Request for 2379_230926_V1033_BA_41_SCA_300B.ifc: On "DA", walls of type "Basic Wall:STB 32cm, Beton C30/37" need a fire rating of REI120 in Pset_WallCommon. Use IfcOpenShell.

First a look at what the model holds.

```python
import ifcopenshell
import ifcopenshell.util.element

model = ifcopenshell.open("2379_230926_V1033_BA_41_SCA_300B.ifc")
print(model.schema)
storey = next(s for s in model.by_type("IfcBuildingStorey") if s.Name == "DA")
walls = [e for e in ifcopenshell.util.element.get_decomposition(storey) if e.is_a("IfcWall")]
seen = {}
for e in walls:
    element_type = ifcopenshell.util.element.get_type(e)
    key = (element_type.Name if element_type != e and element_type else None, ifcopenshell.util.element.get_pset(e, "Pset_WallCommon", "FireRating"))
    seen[key] = seen.get(key, 0) + 1
for (name, value), count in sorted(seen.items(), key=str):
    print(count, "x", name, "|", value)
```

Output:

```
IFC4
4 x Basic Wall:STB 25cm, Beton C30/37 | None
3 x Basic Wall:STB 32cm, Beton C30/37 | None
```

```python
import ifcopenshell
import ifcopenshell.api.pset
import ifcopenshell.util.element

model = ifcopenshell.open("2379_230926_V1033_BA_41_SCA_300B.ifc")

storey = next(s for s in model.by_type("IfcBuildingStorey") if s.Name == "DA")
walls = [e for e in ifcopenshell.util.element.get_decomposition(storey) if e.is_a("IfcWall")]

count = 0
for e in walls:
    element_type = ifcopenshell.util.element.get_type(e)
    if element_type in (None, e) or element_type.Name != "Basic Wall:STB 32cm, Beton C30/37":
        continue
    # add_pset returns the element's existing set when there is one.
    pset = ifcopenshell.api.pset.add_pset(model, product=e, name="Pset_WallCommon")
    ifcopenshell.api.pset.edit_pset(model, pset=pset, properties={"FireRating": "REI120"})
    count += 1

print(count, "walls updated")

model.write("2379_230926_V1033_BA_41_SCA_300B_updated.ifc")
```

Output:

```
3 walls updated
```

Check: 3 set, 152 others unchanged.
